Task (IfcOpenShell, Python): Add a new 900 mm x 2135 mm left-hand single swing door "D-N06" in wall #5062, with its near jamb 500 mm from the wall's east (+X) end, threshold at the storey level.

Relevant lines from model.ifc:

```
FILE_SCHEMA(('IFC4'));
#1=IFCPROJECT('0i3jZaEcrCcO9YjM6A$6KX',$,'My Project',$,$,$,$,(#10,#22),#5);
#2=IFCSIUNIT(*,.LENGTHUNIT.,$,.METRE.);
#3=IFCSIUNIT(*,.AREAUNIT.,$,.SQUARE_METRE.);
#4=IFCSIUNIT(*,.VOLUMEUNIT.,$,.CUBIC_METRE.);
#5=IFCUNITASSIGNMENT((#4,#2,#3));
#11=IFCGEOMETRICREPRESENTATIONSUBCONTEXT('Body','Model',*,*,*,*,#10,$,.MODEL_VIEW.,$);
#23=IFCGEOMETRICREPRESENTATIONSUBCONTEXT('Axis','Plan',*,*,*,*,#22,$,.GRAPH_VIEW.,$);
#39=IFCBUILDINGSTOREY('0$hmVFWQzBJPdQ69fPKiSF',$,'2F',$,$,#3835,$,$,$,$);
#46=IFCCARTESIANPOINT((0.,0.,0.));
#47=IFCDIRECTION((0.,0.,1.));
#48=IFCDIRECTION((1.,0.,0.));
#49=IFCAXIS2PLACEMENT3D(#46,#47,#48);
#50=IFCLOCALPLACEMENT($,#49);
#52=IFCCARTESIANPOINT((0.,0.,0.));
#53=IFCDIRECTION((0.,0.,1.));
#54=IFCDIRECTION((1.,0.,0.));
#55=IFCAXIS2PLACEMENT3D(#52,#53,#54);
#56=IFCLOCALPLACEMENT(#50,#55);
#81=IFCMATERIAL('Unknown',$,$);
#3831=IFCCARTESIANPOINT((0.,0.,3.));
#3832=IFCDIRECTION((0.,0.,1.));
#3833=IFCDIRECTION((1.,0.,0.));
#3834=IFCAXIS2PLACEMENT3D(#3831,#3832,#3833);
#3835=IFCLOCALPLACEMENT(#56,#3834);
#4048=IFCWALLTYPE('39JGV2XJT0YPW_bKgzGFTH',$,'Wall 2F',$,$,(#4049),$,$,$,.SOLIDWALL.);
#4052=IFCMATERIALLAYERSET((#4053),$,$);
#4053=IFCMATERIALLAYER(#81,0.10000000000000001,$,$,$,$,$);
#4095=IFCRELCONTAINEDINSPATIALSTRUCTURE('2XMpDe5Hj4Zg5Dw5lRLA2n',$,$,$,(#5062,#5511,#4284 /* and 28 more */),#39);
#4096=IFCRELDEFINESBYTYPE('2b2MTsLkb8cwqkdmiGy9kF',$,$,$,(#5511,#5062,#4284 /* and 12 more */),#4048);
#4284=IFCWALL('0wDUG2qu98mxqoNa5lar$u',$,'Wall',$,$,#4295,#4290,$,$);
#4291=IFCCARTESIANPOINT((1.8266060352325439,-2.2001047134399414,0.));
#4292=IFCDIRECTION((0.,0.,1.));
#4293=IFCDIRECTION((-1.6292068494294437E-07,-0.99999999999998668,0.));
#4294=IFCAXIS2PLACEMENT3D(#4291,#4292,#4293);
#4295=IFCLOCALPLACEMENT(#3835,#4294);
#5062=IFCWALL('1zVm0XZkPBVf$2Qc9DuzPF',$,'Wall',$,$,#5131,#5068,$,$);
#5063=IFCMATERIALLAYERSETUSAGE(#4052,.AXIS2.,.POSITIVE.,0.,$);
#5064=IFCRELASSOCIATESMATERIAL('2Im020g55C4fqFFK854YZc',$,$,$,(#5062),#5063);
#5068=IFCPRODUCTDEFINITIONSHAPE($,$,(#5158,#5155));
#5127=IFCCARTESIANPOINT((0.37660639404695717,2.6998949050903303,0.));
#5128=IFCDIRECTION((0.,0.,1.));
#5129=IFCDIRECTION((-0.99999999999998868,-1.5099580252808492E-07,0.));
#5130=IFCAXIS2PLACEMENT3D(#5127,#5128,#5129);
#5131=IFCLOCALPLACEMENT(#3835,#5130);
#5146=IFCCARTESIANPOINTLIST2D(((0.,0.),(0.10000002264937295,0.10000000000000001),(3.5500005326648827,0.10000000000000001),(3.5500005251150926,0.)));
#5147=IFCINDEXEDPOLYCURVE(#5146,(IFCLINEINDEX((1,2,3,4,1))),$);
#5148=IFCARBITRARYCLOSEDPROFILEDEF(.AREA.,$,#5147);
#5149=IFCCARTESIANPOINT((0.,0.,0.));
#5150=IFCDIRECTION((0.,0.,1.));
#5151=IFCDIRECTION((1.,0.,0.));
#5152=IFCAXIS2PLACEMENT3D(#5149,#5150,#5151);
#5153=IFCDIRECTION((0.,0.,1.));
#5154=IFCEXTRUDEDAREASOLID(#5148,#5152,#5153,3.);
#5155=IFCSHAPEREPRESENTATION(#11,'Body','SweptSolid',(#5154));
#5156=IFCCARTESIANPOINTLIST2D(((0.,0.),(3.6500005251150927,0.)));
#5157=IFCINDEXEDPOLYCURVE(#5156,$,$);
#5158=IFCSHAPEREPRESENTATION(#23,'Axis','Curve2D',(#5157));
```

```python
import numpy as np
import ifcopenshell
import ifcopenshell.api.feature
import ifcopenshell.api.geometry
import ifcopenshell.api.root
import ifcopenshell.api.spatial
import ifcopenshell.geom
import ifcopenshell.util.element
import ifcopenshell.util.placement
import ifcopenshell.util.representation
import ifcopenshell.util.shape
import ifcopenshell.util.unit

model = ifcopenshell.open("model.ifc")
unit_scale = ifcopenshell.util.unit.calculate_unit_scale(model)
settings = ifcopenshell.geom.settings()


def volume(element):
    """Net volume in cubic metres, openings subtracted."""
    shape = ifcopenshell.geom.create_shape(settings, element)
    return ifcopenshell.util.shape.get_volume(shape.geometry)


wall = model.by_id(5062)
storey = ifcopenshell.util.element.get_container(wall, ifc_class="IfcBuildingStorey")
context = ifcopenshell.util.representation.get_context(model, "Model", "Body", "MODEL_VIEW")
before = volume(wall)

width, height, from_end, sill = 0.9, 2.135, 0.5, 0.0  # metres

# The wall runs along its own X axis, and the end named is its -X end.
wall_shape = ifcopenshell.geom.create_shape(settings, wall)
x, y, z = ifcopenshell.util.shape.get_vertices(wall_shape.geometry).T
start = x.min() + from_end
face, thickness = float(y.min()), float(y.max() - y.min())
wall_matrix = ifcopenshell.util.placement.get_local_placement(wall.ObjectPlacement)
level = ifcopenshell.util.placement.get_local_placement(storey.ObjectPlacement)[2, 3]


def in_wall(x, y):
    """Placement at x, y metres in the wall's axes, at sill height."""
    matrix = wall_matrix.copy()
    matrix[:, 3] = wall_matrix @ np.array([x / unit_scale, y / unit_scale, 0.0, 1.0])
    matrix[2, 3] = level + sill / unit_scale
    return matrix


# Opening: a box that overshoots both wall faces by 50 mm.
opening = ifcopenshell.api.root.create_entity(model, ifc_class="IfcOpeningElement", predefined_type="OPENING")
box = ifcopenshell.api.geometry.add_wall_representation(
    model, context=context, length=width, height=height, thickness=thickness + 0.1
)
ifcopenshell.api.geometry.assign_representation(model, product=opening, representation=box)
ifcopenshell.api.geometry.edit_object_placement(model, product=opening, matrix=in_wall(start, face - 0.05), is_si=False)
ifcopenshell.api.feature.add_feature(model, feature=opening, element=wall)

door = ifcopenshell.api.root.create_entity(model, ifc_class="IfcDoor", name="D-N06", predefined_type="DOOR")
door.OverallWidth, door.OverallHeight = width / unit_scale, height / unit_scale
door.OperationType = "SINGLE_SWING_LEFT"
body = ifcopenshell.api.geometry.add_door_representation(
    model,
    context=context,
    overall_width=door.OverallWidth,
    overall_height=door.OverallHeight,
    operation_type="SINGLE_SWING_LEFT",
    lining_properties={"LiningDepth": thickness / unit_scale, "ThresholdDepth": thickness / unit_scale},
)
ifcopenshell.api.geometry.assign_representation(model, product=door, representation=body)
ifcopenshell.api.spatial.assign_container(model, products=[door], relating_structure=storey)
ifcopenshell.api.feature.add_filling(model, opening=opening, element=door)

# The lining spans the wall, so the door starts at the wall face.
ifcopenshell.api.geometry.edit_object_placement(model, product=door, matrix=in_wall(start, face), is_si=False)

after = volume(wall)

print(f"wall volume {before:.3f} -> {after:.3f} m3")

model.write("model-out.ifc")
```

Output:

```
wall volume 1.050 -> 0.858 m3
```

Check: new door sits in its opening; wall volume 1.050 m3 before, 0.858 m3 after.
